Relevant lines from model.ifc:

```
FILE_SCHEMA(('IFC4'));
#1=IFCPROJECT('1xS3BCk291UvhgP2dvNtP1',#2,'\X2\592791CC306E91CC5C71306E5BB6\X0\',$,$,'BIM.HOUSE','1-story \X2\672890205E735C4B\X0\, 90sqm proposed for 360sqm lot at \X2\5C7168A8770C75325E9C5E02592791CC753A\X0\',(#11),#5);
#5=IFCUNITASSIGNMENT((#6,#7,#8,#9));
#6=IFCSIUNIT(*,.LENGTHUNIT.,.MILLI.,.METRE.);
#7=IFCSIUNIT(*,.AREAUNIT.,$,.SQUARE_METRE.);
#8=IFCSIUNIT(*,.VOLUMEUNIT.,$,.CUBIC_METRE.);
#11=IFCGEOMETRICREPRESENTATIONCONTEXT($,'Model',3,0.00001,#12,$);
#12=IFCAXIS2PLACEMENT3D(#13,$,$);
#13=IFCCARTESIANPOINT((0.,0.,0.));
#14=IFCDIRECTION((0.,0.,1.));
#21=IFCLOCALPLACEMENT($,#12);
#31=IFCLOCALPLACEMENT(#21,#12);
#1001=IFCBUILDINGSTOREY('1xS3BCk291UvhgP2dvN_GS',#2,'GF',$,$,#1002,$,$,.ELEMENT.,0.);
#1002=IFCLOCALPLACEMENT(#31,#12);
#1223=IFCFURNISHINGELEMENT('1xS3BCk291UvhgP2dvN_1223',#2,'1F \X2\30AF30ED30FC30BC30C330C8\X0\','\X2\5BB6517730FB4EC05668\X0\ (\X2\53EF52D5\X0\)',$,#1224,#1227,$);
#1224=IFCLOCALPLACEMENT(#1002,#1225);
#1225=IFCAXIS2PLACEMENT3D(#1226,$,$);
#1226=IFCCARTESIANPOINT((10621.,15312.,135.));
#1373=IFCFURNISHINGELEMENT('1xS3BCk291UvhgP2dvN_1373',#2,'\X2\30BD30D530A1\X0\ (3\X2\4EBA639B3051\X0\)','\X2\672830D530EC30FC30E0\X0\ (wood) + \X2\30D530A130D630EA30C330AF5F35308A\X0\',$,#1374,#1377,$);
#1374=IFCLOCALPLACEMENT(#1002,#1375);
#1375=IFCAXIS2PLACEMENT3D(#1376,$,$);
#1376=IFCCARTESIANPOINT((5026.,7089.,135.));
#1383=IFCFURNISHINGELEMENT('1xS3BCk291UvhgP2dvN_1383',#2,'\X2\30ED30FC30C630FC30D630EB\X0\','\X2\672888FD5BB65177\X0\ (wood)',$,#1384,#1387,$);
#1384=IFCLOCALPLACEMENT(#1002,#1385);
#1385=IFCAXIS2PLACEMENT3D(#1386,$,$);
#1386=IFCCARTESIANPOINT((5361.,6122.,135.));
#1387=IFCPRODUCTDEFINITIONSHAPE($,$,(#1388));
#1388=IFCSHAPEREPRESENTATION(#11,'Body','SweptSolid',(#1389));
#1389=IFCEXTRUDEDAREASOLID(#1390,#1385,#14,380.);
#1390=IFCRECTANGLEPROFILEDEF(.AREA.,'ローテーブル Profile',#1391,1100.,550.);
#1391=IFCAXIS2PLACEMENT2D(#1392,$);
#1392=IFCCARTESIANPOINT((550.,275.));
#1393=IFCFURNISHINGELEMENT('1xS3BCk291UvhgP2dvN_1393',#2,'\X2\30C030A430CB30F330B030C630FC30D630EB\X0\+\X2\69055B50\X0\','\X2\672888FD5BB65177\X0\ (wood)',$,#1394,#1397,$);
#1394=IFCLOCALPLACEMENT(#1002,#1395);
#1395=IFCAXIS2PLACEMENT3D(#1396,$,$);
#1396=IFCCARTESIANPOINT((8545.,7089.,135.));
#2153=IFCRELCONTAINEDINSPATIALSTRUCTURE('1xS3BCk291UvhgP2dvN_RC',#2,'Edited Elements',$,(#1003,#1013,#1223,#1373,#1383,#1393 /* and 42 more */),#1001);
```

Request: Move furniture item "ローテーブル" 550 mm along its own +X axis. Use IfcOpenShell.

```python
import ifcopenshell
import ifcopenshell.api.geometry
import ifcopenshell.util.placement

model = ifcopenshell.open("model.ifc")

item = model.by_guid("1xS3BCk291UvhgP2dvN_1383")
matrix = ifcopenshell.util.placement.get_local_placement(item.ObjectPlacement)
matrix[:3, 3] += matrix[:3, 0] * 550.0
ifcopenshell.api.geometry.edit_object_placement(model, product=item, matrix=matrix, is_si=False)

print(ifcopenshell.util.placement.get_local_placement(item.ObjectPlacement).round(3) + 0.0)

model.write("model_v2.ifc")
```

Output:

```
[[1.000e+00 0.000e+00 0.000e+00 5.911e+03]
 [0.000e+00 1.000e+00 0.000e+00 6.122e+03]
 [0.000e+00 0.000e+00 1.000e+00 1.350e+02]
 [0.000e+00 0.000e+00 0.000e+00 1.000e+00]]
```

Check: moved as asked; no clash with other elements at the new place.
